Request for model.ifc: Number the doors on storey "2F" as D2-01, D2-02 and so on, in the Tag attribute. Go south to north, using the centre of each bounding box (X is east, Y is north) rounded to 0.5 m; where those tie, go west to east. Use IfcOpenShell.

First a look at what the model holds.

```python
import ifcopenshell
import ifcopenshell.util.element
import ifcopenshell.util.placement

model = ifcopenshell.open("model.ifc")
print(model.schema)
storey = next(s for s in model.by_type("IfcBuildingStorey") if s.Name == "2F")
doors = [e for e in ifcopenshell.util.element.get_decomposition(storey) if e.is_a("IfcDoor")]
for e in sorted(doors, key=lambda e: e.id()):
    origin = ifcopenshell.util.placement.get_local_placement(e.ObjectPlacement)[:3, 3]
    print(e.id(), e.Tag, e.Name, origin.round(2) + 0.0, sep=" | ")
```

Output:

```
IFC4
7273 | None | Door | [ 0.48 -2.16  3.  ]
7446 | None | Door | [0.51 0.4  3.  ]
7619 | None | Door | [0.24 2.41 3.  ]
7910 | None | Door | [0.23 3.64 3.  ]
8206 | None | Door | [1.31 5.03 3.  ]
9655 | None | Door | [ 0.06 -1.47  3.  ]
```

```python
import ifcopenshell
import ifcopenshell.geom
import ifcopenshell.util.element
import ifcopenshell.util.shape

model = ifcopenshell.open("model.ifc")
settings = ifcopenshell.geom.settings()
settings.set("use-world-coords", True)


def centre(element):
    shape = ifcopenshell.geom.create_shape(settings, element)
    return ifcopenshell.util.shape.get_bbox_centroid(shape.geometry)


storey = next(s for s in model.by_type("IfcBuildingStorey") if s.Name == "2F")
doors = [e for e in ifcopenshell.util.element.get_decomposition(storey) if e.is_a("IfcDoor")]

# Insertion points can sit at a corner or the storey origin, so sort by the geometry (in metres).
centres = {e: centre(e) for e in doors}
doors.sort(key=lambda e: (round(centres[e][1] / 0.5), centres[e][0]))

for i, e in enumerate(doors, start=1):
    number = f"D2-{i:02d}"
    e.Tag = number
    print(e.id(), number)

model.write("model_rev.ifc")
```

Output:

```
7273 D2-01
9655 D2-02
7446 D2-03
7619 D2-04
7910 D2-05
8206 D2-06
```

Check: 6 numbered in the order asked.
